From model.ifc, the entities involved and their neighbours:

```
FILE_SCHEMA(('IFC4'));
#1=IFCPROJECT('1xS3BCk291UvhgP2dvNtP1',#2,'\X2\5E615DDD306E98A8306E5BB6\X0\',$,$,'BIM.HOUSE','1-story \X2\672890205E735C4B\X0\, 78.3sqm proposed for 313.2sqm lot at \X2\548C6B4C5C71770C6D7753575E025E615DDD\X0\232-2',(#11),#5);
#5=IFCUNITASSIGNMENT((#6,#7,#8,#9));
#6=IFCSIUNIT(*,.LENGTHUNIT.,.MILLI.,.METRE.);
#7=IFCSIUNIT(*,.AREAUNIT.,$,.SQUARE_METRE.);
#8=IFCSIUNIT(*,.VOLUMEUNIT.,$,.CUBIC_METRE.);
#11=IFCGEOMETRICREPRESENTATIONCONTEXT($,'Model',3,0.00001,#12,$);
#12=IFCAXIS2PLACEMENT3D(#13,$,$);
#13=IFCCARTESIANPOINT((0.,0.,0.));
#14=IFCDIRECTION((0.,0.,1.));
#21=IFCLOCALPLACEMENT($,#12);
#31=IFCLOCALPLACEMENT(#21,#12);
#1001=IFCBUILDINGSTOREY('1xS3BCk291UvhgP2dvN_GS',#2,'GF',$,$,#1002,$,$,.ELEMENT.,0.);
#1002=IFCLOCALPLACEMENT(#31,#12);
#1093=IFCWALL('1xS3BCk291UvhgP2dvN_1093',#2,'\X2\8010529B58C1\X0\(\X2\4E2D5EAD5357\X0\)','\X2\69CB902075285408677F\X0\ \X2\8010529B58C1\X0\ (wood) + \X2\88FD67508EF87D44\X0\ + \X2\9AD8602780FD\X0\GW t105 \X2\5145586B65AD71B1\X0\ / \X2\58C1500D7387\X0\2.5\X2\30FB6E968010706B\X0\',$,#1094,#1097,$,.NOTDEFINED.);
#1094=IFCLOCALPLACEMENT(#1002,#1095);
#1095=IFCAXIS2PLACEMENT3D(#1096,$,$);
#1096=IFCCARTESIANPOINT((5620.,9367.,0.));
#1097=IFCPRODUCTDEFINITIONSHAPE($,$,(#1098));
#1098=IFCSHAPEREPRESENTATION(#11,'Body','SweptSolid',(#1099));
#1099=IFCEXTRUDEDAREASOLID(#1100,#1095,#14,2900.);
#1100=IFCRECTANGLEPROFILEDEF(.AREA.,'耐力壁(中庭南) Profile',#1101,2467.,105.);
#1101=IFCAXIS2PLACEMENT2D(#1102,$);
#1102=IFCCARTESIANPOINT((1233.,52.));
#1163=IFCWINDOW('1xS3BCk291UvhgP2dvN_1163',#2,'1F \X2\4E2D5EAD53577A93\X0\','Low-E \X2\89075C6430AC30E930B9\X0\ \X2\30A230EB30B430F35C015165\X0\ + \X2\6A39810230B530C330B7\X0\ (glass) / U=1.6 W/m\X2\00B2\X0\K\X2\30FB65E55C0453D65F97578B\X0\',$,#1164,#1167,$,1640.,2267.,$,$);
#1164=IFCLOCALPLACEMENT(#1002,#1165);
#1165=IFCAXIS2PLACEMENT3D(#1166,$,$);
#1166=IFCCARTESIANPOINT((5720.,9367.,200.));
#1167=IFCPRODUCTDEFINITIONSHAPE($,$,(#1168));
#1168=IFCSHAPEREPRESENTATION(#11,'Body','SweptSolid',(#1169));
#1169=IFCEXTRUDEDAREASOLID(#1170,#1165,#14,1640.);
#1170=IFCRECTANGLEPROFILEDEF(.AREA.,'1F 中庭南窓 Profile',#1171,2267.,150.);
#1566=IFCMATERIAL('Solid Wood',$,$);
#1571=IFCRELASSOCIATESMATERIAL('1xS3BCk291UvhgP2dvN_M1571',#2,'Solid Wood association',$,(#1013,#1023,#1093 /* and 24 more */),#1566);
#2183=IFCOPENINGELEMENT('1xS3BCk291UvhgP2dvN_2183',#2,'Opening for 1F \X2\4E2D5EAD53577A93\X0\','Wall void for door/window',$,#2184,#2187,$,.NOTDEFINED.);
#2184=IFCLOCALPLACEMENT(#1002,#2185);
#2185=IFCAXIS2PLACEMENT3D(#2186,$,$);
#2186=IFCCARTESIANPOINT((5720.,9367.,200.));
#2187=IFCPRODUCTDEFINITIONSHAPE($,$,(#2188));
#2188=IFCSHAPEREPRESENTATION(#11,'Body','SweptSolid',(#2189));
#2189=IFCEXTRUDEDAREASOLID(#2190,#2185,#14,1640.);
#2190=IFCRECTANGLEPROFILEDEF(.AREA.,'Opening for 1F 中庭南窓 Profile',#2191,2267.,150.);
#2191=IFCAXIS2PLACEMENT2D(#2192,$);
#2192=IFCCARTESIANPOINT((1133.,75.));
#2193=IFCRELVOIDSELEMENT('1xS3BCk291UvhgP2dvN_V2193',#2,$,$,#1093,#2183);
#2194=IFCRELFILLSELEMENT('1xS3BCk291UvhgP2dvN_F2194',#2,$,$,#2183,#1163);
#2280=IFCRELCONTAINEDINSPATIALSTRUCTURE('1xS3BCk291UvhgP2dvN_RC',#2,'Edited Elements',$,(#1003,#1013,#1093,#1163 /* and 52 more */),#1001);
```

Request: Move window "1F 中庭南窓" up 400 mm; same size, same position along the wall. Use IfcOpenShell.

```python
import numpy as np
import ifcopenshell
import ifcopenshell.api.geometry
import ifcopenshell.util.placement
import ifcopenshell.util.unit

model = ifcopenshell.open("model.ifc")
unit_scale = ifcopenshell.util.unit.calculate_unit_scale(model)

window = model.by_guid("1xS3BCk291UvhgP2dvN_1163")
opening = window.FillsVoids[0].RelatingOpeningElement
dz = 0.4 / unit_scale

shift = np.array([0.0, 0.0, dz])
# The window is not placed relative to its opening, so move both.
for product in (opening, window):
    matrix = ifcopenshell.util.placement.get_local_placement(product.ObjectPlacement)
    matrix[:3, 3] += shift
    ifcopenshell.api.geometry.edit_object_placement(model, product=product, matrix=matrix, is_si=False)

print(f"moved by {dz * unit_scale:+.3f} m")

model.write("model_edited.ifc")
```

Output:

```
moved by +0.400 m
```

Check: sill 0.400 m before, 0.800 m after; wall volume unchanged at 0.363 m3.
